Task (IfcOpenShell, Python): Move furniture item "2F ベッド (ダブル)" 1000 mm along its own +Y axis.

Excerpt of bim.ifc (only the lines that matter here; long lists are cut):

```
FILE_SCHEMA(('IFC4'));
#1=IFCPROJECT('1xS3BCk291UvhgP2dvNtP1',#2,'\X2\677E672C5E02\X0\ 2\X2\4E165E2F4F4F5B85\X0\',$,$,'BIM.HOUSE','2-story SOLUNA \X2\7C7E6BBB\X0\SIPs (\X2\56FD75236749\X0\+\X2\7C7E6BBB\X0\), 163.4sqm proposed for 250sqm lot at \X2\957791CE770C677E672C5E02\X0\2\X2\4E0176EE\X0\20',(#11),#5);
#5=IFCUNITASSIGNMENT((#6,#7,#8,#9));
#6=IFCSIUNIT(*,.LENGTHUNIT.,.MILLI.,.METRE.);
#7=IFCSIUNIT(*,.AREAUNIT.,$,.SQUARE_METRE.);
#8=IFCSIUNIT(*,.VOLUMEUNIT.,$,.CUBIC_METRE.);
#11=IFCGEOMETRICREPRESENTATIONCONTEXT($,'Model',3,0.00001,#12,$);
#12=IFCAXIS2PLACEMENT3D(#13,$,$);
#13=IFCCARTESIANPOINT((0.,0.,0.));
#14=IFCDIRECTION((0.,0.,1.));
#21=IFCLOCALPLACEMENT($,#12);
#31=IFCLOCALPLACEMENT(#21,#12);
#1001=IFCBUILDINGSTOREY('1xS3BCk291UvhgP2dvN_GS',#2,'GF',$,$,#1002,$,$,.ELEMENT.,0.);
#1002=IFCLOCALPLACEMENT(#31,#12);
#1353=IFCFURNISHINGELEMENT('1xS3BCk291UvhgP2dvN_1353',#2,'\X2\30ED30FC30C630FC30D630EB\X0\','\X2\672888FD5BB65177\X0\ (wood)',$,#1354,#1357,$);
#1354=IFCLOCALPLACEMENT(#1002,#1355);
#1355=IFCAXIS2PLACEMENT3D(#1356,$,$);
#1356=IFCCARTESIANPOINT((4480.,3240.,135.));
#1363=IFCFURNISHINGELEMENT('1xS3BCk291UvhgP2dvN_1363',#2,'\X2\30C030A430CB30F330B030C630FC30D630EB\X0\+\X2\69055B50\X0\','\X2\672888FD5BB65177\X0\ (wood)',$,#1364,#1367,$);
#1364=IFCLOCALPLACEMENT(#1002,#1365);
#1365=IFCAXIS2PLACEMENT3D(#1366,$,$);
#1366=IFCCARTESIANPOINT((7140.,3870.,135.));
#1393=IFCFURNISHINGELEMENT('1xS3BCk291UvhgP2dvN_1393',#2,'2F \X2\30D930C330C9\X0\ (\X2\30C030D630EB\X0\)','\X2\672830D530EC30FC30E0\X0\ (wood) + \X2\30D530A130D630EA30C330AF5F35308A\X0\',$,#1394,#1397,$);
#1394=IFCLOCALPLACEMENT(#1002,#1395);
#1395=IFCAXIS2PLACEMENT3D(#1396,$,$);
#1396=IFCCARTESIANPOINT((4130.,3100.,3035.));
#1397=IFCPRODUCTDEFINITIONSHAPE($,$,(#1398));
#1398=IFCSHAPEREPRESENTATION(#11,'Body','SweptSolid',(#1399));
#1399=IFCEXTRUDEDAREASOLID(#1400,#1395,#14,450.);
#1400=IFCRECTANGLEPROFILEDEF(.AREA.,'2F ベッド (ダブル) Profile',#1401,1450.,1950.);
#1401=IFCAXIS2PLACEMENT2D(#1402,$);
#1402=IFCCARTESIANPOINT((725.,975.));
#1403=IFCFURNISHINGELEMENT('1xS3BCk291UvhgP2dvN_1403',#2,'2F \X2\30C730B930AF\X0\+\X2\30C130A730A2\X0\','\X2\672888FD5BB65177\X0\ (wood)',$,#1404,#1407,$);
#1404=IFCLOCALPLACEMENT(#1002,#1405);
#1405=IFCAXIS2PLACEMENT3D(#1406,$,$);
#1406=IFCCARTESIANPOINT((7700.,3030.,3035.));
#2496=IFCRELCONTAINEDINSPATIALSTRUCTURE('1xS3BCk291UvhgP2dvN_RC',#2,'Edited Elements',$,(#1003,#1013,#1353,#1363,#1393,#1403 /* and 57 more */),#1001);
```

```python
import ifcopenshell
import ifcopenshell.api.geometry
import ifcopenshell.util.placement
import ifcopenshell.util.unit

model = ifcopenshell.open("bim.ifc")
unit_scale = ifcopenshell.util.unit.calculate_unit_scale(model)

item = model.by_id(1393)
matrix = ifcopenshell.util.placement.get_local_placement(item.ObjectPlacement)
matrix[:3, 3] += matrix[:3, 1] * 1 / unit_scale
ifcopenshell.api.geometry.edit_object_placement(model, product=item, matrix=matrix, is_si=False)

print(ifcopenshell.util.placement.get_local_placement(item.ObjectPlacement).round(3) + 0.0)

model.write("bim_v2.ifc")
```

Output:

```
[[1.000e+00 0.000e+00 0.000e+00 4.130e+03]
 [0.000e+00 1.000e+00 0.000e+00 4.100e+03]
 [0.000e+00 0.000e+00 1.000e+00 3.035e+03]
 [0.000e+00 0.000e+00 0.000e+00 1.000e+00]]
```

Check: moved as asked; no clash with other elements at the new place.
